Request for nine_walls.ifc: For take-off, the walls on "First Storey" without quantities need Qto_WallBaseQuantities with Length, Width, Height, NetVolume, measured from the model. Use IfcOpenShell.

First a look at what the model holds.

```python
import ifcopenshell
import ifcopenshell.util.element
import ifcopenshell.util.unit

model = ifcopenshell.open("nine_walls.ifc")
print(model.schema)
for unit_type in ("LENGTHUNIT", "AREAUNIT", "VOLUMEUNIT"):
    print(unit_type, ifcopenshell.util.unit.calculate_unit_scale(model, unit_type))
storey = next(s for s in model.by_type("IfcBuildingStorey") if s.Name == "First Storey")
walls = [e for e in ifcopenshell.util.element.get_decomposition(storey) if e.is_a("IfcWall")]
for e in sorted(walls, key=lambda e: e.id()):
    print(e.id(), e.is_a(), e.Name, list(ifcopenshell.util.element.get_psets(e, qtos_only=True)), sep=" | ")
```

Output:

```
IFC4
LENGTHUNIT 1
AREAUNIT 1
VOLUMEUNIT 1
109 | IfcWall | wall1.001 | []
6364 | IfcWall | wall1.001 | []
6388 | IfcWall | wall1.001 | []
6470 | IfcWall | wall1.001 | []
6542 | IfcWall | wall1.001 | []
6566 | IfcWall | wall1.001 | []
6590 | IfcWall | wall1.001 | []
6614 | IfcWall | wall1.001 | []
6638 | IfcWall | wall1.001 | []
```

```python
import ifcopenshell
import ifcopenshell.api.pset
import ifcopenshell.geom
import ifcopenshell.util.element
import ifcopenshell.util.shape
import ifcopenshell.util.unit

model = ifcopenshell.open("nine_walls.ifc")
unit_scale = ifcopenshell.util.unit.calculate_unit_scale(model)
volume_scale = ifcopenshell.util.unit.calculate_unit_scale(model, "VOLUMEUNIT")
settings = ifcopenshell.geom.settings()

storey = next(s for s in model.by_type("IfcBuildingStorey") if s.Name == "First Storey")
walls = [e for e in ifcopenshell.util.element.get_decomposition(storey) if e.is_a("IfcWall")]

for e in sorted(walls, key=lambda e: e.id()):
    if ifcopenshell.util.element.get_psets(e, qtos_only=True, should_inherit=False):
        continue
    # Geometry comes back in metres, in the element's own axes.
    shape = ifcopenshell.geom.create_shape(settings, e)
    values = {
        "Length": ifcopenshell.util.shape.get_x(shape.geometry) / unit_scale,
        "Width": ifcopenshell.util.shape.get_y(shape.geometry) / unit_scale,
        "Height": ifcopenshell.util.shape.get_z(shape.geometry) / unit_scale,
        "NetVolume": ifcopenshell.util.shape.get_volume(shape.geometry) / volume_scale,
    }
    qto = ifcopenshell.api.pset.add_qto(model, product=e, name="Qto_WallBaseQuantities")
    ifcopenshell.api.pset.edit_qto(model, qto=qto, properties=values)
    print(e.id(), {k: round(v, 3) for k, v in values.items()})

model.write("nine_walls_edited.ifc")
```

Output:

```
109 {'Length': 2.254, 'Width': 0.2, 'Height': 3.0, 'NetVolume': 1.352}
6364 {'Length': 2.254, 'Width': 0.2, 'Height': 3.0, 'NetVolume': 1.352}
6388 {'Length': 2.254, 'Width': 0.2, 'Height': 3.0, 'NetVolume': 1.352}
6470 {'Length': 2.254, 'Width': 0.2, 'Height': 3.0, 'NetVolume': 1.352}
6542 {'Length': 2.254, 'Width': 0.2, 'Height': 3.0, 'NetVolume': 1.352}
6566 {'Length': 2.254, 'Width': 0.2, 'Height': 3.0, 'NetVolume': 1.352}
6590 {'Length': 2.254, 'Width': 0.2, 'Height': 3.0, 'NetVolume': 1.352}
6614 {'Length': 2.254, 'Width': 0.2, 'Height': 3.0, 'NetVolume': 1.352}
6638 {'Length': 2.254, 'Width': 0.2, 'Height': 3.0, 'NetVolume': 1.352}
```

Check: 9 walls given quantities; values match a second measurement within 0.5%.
